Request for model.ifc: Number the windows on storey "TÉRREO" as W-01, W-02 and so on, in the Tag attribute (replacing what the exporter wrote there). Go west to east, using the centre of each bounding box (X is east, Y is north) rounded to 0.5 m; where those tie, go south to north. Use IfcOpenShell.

First a look at what the model holds.

```python
import ifcopenshell
import ifcopenshell.util.element
import ifcopenshell.util.placement

model = ifcopenshell.open("model.ifc")
print(model.schema)
storey = next(s for s in model.by_type("IfcBuildingStorey") if s.Name == "TÉRREO")
windows = [e for e in ifcopenshell.util.element.get_decomposition(storey) if e.is_a("IfcWindow")]
for e in sorted(windows, key=lambda e: e.id()):
    origin = ifcopenshell.util.placement.get_local_placement(e.ObjectPlacement)[:3, 3]
    print(e.id(), e.Tag, e.Name, origin.round(2) + 0.0, sep=" | ")
```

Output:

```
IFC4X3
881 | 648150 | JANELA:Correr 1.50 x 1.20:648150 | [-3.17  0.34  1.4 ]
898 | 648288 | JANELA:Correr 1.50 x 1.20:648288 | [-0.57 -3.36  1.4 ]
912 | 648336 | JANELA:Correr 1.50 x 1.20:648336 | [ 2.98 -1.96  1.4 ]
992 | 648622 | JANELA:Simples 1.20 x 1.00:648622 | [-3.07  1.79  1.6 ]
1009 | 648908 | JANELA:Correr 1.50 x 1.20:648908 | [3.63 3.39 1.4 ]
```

```python
import ifcopenshell
import ifcopenshell.geom
import ifcopenshell.util.element
import ifcopenshell.util.shape

model = ifcopenshell.open("model.ifc")
settings = ifcopenshell.geom.settings()
settings.set("use-world-coords", True)


def centre(element):
    shape = ifcopenshell.geom.create_shape(settings, element)
    return ifcopenshell.util.shape.get_bbox_centroid(shape.geometry)


storey = next(s for s in model.by_type("IfcBuildingStorey") if s.Name == "TÉRREO")
windows = [e for e in ifcopenshell.util.element.get_decomposition(storey) if e.is_a("IfcWindow")]

# Insertion points can sit at a corner or the storey origin, so sort by the geometry (in metres).
centres = {e: centre(e) for e in windows}
windows.sort(key=lambda e: (round(centres[e][0] / 0.5), centres[e][1]))

for i, e in enumerate(windows, start=1):
    number = f"W-{i:02d}"
    e.Tag = number
    print(e.id(), number)

model.write("model_edited.ifc")
```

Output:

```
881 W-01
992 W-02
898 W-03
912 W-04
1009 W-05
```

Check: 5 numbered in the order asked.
